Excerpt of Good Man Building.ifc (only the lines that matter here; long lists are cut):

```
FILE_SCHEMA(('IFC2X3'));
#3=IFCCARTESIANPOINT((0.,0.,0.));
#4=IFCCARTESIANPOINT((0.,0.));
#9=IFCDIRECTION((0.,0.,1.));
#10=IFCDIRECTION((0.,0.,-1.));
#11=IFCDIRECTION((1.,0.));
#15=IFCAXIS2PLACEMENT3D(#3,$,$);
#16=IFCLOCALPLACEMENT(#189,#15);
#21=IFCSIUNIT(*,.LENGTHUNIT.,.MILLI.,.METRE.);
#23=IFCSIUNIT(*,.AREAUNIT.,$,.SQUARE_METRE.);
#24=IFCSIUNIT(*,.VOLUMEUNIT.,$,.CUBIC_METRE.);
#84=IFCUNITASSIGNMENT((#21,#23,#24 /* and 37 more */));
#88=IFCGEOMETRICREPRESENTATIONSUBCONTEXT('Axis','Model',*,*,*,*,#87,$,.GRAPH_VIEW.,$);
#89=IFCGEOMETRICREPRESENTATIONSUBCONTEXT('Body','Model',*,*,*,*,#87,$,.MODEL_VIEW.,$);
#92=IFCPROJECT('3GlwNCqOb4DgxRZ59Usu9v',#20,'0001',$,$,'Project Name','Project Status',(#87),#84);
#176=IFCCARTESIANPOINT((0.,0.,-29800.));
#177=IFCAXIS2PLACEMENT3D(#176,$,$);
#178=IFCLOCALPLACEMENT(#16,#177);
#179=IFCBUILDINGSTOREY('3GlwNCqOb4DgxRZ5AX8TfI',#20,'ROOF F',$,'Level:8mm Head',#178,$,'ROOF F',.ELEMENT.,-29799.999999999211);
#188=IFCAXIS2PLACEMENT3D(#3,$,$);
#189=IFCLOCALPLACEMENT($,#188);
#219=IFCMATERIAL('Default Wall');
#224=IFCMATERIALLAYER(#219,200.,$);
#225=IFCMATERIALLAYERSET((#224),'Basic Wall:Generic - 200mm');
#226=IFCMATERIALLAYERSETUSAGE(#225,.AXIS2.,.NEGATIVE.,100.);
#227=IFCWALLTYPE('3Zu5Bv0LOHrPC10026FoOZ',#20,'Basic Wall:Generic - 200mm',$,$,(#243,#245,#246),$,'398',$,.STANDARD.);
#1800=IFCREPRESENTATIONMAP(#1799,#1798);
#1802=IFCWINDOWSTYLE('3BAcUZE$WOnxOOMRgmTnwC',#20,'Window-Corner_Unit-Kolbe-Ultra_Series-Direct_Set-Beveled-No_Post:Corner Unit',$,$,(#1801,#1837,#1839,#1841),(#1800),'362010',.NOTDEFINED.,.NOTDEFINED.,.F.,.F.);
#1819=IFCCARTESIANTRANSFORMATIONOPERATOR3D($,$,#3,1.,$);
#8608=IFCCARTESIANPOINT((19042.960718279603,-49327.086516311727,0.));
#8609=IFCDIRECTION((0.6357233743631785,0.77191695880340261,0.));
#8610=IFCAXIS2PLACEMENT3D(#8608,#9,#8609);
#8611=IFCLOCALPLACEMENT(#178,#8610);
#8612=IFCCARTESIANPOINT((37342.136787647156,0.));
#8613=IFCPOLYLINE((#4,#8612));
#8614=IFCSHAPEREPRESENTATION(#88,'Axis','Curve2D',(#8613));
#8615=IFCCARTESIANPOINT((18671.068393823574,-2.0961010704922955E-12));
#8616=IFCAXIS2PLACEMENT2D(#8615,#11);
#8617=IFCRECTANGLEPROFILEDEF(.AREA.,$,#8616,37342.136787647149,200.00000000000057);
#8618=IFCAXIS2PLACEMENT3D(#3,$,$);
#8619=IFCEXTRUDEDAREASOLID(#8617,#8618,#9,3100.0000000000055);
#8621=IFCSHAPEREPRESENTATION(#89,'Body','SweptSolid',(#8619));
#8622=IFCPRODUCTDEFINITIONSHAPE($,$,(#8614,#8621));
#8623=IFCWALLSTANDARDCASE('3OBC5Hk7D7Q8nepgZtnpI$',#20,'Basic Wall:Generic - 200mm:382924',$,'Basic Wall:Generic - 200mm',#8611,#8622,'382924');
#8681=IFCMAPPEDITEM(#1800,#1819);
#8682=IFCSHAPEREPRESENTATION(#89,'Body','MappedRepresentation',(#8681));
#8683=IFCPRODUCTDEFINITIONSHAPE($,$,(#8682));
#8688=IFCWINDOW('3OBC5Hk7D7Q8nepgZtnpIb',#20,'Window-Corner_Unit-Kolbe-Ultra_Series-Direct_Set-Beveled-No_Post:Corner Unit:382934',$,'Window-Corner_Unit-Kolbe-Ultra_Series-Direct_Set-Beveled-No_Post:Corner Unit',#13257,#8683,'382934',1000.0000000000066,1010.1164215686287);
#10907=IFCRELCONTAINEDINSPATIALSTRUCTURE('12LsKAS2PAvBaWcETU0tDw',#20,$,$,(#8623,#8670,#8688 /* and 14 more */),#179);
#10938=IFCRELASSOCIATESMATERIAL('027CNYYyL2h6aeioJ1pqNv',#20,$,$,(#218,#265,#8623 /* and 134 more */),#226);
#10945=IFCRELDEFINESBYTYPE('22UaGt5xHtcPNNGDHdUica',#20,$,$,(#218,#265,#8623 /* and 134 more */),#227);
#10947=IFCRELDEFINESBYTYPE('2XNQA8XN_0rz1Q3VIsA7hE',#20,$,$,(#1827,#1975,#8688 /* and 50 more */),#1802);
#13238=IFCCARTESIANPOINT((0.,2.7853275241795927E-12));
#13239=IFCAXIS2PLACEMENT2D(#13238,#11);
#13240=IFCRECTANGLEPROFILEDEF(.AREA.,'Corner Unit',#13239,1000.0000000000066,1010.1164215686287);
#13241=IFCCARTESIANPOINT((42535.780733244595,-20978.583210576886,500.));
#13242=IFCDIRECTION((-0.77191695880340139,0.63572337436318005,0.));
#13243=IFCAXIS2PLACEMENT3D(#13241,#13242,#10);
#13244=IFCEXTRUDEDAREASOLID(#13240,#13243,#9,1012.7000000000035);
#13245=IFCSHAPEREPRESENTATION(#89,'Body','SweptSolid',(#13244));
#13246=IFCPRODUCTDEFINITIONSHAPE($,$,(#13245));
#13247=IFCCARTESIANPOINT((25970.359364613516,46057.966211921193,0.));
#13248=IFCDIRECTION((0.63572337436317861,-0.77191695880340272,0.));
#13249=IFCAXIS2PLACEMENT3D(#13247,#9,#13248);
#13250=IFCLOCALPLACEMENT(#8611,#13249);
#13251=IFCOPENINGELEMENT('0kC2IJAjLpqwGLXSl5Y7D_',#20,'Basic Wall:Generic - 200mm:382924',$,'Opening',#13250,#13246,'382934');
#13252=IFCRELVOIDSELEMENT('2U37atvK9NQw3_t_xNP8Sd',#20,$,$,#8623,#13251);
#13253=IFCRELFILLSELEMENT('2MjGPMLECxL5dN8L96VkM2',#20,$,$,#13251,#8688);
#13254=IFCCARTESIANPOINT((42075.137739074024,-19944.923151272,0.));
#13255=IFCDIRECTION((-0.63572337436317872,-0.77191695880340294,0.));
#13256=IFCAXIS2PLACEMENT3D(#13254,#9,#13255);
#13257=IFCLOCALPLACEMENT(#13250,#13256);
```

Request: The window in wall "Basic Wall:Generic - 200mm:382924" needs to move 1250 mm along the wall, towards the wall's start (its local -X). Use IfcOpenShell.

```python
import ifcopenshell
import ifcopenshell.api.geometry
import ifcopenshell.util.placement

model = ifcopenshell.open("Good Man Building.ifc")

window = model.by_guid("3OBC5Hk7D7Q8nepgZtnpIb")
opening = window.FillsVoids[0].RelatingOpeningElement
wall = opening.VoidsElements[0].RelatingBuildingElement

wall_matrix = ifcopenshell.util.placement.get_local_placement(wall.ObjectPlacement)
shift = wall_matrix[:3, 0] * -1250.0
before = ifcopenshell.util.placement.get_local_placement(window.ObjectPlacement)[:3, 3].copy()

# The window is placed relative to its opening, so it follows when the opening moves.
matrix = ifcopenshell.util.placement.get_local_placement(opening.ObjectPlacement)
matrix[:3, 3] += shift
ifcopenshell.api.geometry.edit_object_placement(
    model, product=opening, matrix=matrix, is_si=False, should_transform_children=True
)

after = ifcopenshell.util.placement.get_local_placement(window.ObjectPlacement)[:3, 3]
print("window moved by", (after - before).round(3) + 0.0)

model.write("Good Man Building_edited.ifc")
```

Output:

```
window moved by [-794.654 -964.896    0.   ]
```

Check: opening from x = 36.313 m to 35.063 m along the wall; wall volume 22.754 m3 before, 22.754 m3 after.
